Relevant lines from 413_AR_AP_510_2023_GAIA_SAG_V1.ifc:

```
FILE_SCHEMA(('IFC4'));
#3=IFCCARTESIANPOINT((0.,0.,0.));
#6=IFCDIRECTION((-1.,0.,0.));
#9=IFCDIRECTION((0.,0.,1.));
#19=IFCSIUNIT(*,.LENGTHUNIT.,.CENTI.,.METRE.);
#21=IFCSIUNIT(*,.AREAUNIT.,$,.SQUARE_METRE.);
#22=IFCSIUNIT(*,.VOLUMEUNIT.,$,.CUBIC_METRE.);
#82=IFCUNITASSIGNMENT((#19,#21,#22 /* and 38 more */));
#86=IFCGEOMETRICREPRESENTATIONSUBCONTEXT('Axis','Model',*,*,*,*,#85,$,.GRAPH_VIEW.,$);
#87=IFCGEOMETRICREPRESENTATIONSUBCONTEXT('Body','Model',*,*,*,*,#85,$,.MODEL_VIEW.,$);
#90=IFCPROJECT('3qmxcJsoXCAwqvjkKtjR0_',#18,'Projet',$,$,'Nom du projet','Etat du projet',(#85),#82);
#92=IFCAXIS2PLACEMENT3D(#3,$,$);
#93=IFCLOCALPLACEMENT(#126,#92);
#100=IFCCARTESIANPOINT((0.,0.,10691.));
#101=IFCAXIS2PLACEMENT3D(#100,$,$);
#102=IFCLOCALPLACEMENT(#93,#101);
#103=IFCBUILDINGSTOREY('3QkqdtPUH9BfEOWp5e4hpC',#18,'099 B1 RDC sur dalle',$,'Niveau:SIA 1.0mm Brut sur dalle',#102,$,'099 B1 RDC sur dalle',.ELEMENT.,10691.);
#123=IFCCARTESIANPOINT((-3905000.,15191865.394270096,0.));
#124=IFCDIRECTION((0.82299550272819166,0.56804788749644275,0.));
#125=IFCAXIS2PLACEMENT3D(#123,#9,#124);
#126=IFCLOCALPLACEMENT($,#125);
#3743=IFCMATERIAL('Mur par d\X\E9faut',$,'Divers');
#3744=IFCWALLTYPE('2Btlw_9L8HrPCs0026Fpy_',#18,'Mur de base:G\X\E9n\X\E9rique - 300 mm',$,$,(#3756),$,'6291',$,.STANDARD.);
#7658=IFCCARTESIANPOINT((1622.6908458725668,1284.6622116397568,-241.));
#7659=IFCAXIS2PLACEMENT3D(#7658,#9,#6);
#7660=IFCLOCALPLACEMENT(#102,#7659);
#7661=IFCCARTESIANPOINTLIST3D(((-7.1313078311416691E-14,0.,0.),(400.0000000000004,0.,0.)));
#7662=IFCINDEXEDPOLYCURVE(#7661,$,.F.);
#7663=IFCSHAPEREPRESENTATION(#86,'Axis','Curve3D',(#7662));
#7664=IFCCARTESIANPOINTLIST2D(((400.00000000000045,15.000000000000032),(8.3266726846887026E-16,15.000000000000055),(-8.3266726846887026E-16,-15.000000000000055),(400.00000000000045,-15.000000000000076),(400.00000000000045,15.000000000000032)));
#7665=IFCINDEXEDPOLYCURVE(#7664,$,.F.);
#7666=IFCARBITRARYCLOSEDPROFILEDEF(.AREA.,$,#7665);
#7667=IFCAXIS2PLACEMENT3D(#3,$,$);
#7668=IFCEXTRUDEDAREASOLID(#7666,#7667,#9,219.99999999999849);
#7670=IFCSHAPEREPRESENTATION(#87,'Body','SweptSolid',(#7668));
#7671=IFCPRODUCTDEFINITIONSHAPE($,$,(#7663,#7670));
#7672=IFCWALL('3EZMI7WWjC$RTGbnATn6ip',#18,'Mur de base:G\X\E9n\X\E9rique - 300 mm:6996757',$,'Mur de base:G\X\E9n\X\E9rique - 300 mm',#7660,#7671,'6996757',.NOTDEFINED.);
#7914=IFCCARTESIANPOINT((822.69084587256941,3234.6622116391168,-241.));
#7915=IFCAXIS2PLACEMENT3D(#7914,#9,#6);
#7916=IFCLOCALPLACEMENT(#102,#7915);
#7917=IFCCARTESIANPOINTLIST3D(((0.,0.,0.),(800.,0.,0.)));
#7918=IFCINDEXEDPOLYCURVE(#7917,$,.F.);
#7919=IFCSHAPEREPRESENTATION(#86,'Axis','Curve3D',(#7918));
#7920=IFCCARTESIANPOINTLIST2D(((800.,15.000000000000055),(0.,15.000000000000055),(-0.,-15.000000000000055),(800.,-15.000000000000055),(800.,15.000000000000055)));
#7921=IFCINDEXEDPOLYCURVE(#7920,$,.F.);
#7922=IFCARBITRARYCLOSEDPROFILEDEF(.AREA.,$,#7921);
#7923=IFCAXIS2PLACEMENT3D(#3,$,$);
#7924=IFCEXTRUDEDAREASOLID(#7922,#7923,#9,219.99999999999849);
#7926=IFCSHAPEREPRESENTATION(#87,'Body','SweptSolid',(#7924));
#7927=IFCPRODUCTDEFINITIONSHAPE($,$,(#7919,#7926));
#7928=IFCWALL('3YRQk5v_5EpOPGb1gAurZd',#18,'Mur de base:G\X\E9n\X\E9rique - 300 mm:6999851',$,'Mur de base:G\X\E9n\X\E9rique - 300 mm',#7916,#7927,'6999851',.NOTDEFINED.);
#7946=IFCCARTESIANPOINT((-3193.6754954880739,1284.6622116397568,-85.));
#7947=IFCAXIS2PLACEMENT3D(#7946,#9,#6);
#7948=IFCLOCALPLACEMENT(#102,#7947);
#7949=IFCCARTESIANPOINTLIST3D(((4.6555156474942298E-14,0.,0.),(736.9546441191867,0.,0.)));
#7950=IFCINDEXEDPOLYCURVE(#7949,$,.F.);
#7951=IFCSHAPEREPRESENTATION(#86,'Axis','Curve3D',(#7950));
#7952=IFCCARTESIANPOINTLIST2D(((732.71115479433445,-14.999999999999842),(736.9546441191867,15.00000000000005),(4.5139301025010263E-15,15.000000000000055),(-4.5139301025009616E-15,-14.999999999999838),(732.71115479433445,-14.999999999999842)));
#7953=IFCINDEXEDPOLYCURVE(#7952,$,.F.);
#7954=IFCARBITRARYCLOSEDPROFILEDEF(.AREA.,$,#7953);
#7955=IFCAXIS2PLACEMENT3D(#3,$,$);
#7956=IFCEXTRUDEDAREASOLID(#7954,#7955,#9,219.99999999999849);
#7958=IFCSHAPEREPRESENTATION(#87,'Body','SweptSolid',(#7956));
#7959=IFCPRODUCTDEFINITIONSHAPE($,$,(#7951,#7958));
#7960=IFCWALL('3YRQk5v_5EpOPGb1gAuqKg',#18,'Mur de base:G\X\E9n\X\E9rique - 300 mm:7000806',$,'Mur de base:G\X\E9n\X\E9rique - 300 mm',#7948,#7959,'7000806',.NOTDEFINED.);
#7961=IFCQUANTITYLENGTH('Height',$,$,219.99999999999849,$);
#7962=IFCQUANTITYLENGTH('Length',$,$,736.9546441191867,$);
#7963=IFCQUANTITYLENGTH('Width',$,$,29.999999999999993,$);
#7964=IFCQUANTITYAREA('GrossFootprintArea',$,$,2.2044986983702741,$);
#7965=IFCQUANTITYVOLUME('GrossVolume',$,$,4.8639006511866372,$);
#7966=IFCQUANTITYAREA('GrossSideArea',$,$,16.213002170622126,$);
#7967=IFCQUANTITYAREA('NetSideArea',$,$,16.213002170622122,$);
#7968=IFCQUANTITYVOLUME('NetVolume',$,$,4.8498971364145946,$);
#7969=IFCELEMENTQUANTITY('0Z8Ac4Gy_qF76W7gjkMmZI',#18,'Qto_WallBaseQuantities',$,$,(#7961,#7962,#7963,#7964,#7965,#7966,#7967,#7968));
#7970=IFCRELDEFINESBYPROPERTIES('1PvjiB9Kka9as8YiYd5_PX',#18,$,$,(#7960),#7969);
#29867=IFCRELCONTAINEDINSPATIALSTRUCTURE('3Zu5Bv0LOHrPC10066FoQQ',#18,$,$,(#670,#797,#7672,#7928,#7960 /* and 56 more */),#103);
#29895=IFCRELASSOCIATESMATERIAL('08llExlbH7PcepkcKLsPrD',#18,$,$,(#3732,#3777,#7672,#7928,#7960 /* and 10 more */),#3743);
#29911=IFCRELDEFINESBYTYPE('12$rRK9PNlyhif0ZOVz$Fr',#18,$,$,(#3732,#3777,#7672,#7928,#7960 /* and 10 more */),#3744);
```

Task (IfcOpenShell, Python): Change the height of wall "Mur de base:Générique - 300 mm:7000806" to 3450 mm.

```python
import ifcopenshell
import ifcopenshell.api.pset
import ifcopenshell.geom
import ifcopenshell.util.element
import ifcopenshell.util.representation
import ifcopenshell.util.shape
import ifcopenshell.util.unit

model = ifcopenshell.open("413_AR_AP_510_2023_GAIA_SAG_V1.ifc")
unit_scale = ifcopenshell.util.unit.calculate_unit_scale(model)
area_scale = ifcopenshell.util.unit.calculate_unit_scale(model, "AREAUNIT")
volume_scale = ifcopenshell.util.unit.calculate_unit_scale(model, "VOLUMEUNIT")
settings = ifcopenshell.geom.settings()


def volume(element):
    """Net volume in cubic metres, openings subtracted."""
    shape = ifcopenshell.geom.create_shape(settings, element)
    return ifcopenshell.util.shape.get_volume(shape.geometry)


wall = model.by_id(7960)
before = volume(wall)

body = ifcopenshell.util.representation.get_representation(wall, "Model", "Body")
solid = body.Items[0]
old_height = solid.Depth
solid.Depth = 3.45 / unit_scale
after = volume(wall)
thickness = 0.3  # wall thickness in metres

# Update the stored height, areas and volumes.
qto = model.by_id(ifcopenshell.util.element.get_pset(wall, "Qto_WallBaseQuantities", should_inherit=False)["id"])
ifcopenshell.api.pset.edit_qto(model, qto=qto, properties={
    "Height": solid.Depth,
    "GrossVolume": ifcopenshell.util.element.get_pset(wall, "Qto_WallBaseQuantities", "GrossVolume") * solid.Depth / old_height,
    "GrossSideArea": ifcopenshell.util.element.get_pset(wall, "Qto_WallBaseQuantities", "GrossSideArea") * solid.Depth / old_height,
    "NetSideArea": after / thickness / area_scale,
    "NetVolume": after / volume_scale,
})

print(f"height {old_height:g} -> {solid.Depth:g}, volume {before:.3f} -> {after:.3f} m3")

model.write("413_AR_AP_510_2023_GAIA_SAG_V1_rev.ifc")
```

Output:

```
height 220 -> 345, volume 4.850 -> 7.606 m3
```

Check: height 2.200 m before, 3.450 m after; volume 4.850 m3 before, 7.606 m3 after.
